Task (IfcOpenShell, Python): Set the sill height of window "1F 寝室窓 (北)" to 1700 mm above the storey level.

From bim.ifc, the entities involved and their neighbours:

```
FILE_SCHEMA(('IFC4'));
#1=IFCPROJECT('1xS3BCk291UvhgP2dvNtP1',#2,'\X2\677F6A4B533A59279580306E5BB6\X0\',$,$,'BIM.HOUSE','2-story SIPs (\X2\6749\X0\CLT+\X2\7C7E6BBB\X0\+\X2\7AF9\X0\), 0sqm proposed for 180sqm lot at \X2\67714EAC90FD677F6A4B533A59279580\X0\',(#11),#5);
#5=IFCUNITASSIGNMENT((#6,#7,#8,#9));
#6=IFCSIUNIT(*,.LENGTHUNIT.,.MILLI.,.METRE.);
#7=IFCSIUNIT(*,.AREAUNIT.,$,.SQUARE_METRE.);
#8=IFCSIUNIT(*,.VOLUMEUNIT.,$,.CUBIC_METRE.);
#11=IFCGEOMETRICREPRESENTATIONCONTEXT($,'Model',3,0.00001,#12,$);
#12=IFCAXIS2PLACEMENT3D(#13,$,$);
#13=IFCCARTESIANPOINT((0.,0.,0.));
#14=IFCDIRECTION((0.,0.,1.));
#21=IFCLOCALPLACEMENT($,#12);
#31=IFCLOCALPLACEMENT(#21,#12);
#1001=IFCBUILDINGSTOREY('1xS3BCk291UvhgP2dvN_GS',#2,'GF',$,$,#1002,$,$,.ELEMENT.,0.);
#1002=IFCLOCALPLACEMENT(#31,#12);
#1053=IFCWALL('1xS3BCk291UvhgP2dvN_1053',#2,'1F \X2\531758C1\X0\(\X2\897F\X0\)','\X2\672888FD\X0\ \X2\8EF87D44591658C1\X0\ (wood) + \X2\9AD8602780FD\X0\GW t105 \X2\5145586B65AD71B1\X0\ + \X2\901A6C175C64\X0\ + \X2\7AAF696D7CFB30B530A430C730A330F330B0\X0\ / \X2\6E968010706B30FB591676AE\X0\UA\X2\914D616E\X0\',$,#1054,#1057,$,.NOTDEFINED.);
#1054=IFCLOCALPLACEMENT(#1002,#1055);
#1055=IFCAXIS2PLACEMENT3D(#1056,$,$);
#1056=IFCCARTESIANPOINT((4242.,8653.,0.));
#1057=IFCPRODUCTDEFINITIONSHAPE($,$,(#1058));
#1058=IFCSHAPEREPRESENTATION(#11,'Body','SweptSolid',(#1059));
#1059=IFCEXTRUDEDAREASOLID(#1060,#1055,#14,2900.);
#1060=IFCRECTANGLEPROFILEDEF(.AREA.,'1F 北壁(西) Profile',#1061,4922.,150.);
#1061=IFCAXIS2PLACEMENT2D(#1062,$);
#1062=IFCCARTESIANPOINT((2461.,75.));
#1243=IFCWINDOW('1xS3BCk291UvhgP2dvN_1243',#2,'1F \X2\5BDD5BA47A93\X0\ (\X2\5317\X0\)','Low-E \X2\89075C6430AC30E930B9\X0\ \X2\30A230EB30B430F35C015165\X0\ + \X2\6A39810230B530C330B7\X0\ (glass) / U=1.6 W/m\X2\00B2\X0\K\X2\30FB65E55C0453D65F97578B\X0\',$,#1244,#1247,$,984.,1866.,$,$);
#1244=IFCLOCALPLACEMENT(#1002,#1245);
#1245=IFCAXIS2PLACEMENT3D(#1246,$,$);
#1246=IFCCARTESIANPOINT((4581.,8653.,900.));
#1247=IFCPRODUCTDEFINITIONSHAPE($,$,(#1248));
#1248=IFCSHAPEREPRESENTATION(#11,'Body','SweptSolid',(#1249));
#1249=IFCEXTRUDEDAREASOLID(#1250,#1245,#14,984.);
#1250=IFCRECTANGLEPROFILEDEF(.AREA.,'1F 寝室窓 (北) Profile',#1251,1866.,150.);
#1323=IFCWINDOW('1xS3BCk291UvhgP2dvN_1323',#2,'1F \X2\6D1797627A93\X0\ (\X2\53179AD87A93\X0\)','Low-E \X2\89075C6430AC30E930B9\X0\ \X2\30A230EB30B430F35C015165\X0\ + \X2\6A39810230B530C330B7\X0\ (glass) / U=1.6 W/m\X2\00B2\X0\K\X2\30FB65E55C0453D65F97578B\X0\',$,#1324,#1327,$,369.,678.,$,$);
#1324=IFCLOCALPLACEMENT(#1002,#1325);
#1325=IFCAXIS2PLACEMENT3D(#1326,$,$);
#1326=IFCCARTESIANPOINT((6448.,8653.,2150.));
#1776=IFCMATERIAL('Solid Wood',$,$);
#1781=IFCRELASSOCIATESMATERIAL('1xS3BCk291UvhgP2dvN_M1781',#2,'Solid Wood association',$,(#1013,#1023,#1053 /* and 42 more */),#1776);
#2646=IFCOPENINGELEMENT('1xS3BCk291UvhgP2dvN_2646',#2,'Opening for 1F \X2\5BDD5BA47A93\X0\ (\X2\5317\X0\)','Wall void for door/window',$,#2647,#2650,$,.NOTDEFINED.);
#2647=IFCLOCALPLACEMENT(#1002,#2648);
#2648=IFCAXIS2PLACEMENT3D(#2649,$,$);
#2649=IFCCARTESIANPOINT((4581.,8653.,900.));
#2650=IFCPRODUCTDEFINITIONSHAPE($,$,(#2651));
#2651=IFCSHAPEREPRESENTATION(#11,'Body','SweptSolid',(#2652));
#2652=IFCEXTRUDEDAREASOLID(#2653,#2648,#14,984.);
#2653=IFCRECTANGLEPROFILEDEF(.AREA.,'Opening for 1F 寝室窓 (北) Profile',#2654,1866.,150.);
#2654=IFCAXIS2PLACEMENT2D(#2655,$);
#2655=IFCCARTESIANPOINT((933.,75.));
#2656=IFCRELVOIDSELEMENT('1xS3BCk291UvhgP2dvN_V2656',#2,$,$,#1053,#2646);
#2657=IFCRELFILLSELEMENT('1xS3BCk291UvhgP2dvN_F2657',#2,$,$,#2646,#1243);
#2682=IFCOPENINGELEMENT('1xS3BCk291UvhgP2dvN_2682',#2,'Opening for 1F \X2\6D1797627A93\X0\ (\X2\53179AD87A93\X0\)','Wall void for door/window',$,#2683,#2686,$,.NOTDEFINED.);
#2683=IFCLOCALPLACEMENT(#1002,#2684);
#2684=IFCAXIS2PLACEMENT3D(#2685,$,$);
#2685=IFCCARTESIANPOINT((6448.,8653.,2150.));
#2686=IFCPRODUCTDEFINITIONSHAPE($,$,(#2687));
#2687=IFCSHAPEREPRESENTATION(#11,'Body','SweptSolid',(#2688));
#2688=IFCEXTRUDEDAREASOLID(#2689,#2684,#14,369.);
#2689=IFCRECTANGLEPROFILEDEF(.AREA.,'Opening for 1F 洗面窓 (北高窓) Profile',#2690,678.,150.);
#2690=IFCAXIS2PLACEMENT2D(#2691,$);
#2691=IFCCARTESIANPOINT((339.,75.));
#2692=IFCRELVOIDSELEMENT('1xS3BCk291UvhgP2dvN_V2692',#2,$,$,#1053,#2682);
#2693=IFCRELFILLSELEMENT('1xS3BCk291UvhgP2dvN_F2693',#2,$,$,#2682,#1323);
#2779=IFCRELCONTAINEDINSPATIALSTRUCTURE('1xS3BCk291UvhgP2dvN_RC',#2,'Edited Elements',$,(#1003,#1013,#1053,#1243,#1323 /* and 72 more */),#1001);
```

```python
import numpy as np
import ifcopenshell
import ifcopenshell.api.geometry
import ifcopenshell.geom
import ifcopenshell.util.element
import ifcopenshell.util.placement
import ifcopenshell.util.shape
import ifcopenshell.util.unit

model = ifcopenshell.open("bim.ifc")
unit_scale = ifcopenshell.util.unit.calculate_unit_scale(model)

window = model.by_guid("1xS3BCk291UvhgP2dvN_1243")
opening = window.FillsVoids[0].RelatingOpeningElement
storey = ifcopenshell.util.element.get_container(window, ifc_class="IfcBuildingStorey")
level = ifcopenshell.util.placement.get_local_placement(storey.ObjectPlacement)[2, 3]

# The opening's origin need not be at the sill, so measure its lowest point.
shape = ifcopenshell.geom.create_shape(ifcopenshell.geom.settings(), opening)
bottom = ifcopenshell.util.shape.get_shape_bottom_elevation(shape, shape.geometry) / unit_scale
dz = level + 1.7 / unit_scale - bottom

shift = np.array([0.0, 0.0, dz])
# The window is not placed relative to its opening, so move both.
for product in (opening, window):
    matrix = ifcopenshell.util.placement.get_local_placement(product.ObjectPlacement)
    matrix[:3, 3] += shift
    ifcopenshell.api.geometry.edit_object_placement(model, product=product, matrix=matrix, is_si=False)

print(f"moved by {dz * unit_scale:+.3f} m")

model.write("bim_v2.ifc")
```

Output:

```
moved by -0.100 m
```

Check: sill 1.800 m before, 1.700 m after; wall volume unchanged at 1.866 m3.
